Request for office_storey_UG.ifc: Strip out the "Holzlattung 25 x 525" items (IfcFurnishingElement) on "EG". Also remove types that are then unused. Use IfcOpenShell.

First a look at what the model holds.

```python
import ifcopenshell
import ifcopenshell.util.element

model = ifcopenshell.open("office_storey_UG.ifc")
print(model.schema)
storey = next(s for s in model.by_type("IfcBuildingStorey") if s.Name == "EG")
furniture = [e for e in ifcopenshell.util.element.get_decomposition(storey) if e.is_a("IfcFurnishingElement")]
seen = {}
for e in furniture:
    element_type = ifcopenshell.util.element.get_type(e)
    name = element_type.Name if element_type not in (None, e) else None
    seen[name] = seen.get(name, 0) + 1
for name, count in sorted(seen.items(), key=str):
    print(count, "x", name)
```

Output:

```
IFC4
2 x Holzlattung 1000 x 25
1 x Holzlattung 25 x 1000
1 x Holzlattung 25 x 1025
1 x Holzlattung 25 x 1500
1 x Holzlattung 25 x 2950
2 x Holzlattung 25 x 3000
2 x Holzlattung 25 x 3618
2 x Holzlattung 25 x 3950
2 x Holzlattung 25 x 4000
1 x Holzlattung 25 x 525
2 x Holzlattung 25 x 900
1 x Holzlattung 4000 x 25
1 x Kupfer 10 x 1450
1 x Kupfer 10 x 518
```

```python
import ifcopenshell
import ifcopenshell.api.root
import ifcopenshell.util.element

model = ifcopenshell.open("office_storey_UG.ifc")

storey = next(s for s in model.by_type("IfcBuildingStorey") if s.Name == "EG")
furniture = [e for e in ifcopenshell.util.element.get_decomposition(storey) if e.is_a("IfcFurnishingElement")]
targets = [e for e in furniture if (t := ifcopenshell.util.element.get_type(e)) not in (None, e) and t.Name == "Holzlattung 25 x 525"]
types = {ifcopenshell.util.element.get_type(e) for e in targets} - {None, *targets}

for e in targets:
    ifcopenshell.api.root.remove_product(model, product=e)
print(len(targets), "removed")

unused = [t for t in types if not ifcopenshell.util.element.get_types(t)]
for t in unused:
    ifcopenshell.api.root.remove_product(model, product=t)
print(len(unused), "unused types removed")

model.write("office_storey_UG_v2.ifc")
```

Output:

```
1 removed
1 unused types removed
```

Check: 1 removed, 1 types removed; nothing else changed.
